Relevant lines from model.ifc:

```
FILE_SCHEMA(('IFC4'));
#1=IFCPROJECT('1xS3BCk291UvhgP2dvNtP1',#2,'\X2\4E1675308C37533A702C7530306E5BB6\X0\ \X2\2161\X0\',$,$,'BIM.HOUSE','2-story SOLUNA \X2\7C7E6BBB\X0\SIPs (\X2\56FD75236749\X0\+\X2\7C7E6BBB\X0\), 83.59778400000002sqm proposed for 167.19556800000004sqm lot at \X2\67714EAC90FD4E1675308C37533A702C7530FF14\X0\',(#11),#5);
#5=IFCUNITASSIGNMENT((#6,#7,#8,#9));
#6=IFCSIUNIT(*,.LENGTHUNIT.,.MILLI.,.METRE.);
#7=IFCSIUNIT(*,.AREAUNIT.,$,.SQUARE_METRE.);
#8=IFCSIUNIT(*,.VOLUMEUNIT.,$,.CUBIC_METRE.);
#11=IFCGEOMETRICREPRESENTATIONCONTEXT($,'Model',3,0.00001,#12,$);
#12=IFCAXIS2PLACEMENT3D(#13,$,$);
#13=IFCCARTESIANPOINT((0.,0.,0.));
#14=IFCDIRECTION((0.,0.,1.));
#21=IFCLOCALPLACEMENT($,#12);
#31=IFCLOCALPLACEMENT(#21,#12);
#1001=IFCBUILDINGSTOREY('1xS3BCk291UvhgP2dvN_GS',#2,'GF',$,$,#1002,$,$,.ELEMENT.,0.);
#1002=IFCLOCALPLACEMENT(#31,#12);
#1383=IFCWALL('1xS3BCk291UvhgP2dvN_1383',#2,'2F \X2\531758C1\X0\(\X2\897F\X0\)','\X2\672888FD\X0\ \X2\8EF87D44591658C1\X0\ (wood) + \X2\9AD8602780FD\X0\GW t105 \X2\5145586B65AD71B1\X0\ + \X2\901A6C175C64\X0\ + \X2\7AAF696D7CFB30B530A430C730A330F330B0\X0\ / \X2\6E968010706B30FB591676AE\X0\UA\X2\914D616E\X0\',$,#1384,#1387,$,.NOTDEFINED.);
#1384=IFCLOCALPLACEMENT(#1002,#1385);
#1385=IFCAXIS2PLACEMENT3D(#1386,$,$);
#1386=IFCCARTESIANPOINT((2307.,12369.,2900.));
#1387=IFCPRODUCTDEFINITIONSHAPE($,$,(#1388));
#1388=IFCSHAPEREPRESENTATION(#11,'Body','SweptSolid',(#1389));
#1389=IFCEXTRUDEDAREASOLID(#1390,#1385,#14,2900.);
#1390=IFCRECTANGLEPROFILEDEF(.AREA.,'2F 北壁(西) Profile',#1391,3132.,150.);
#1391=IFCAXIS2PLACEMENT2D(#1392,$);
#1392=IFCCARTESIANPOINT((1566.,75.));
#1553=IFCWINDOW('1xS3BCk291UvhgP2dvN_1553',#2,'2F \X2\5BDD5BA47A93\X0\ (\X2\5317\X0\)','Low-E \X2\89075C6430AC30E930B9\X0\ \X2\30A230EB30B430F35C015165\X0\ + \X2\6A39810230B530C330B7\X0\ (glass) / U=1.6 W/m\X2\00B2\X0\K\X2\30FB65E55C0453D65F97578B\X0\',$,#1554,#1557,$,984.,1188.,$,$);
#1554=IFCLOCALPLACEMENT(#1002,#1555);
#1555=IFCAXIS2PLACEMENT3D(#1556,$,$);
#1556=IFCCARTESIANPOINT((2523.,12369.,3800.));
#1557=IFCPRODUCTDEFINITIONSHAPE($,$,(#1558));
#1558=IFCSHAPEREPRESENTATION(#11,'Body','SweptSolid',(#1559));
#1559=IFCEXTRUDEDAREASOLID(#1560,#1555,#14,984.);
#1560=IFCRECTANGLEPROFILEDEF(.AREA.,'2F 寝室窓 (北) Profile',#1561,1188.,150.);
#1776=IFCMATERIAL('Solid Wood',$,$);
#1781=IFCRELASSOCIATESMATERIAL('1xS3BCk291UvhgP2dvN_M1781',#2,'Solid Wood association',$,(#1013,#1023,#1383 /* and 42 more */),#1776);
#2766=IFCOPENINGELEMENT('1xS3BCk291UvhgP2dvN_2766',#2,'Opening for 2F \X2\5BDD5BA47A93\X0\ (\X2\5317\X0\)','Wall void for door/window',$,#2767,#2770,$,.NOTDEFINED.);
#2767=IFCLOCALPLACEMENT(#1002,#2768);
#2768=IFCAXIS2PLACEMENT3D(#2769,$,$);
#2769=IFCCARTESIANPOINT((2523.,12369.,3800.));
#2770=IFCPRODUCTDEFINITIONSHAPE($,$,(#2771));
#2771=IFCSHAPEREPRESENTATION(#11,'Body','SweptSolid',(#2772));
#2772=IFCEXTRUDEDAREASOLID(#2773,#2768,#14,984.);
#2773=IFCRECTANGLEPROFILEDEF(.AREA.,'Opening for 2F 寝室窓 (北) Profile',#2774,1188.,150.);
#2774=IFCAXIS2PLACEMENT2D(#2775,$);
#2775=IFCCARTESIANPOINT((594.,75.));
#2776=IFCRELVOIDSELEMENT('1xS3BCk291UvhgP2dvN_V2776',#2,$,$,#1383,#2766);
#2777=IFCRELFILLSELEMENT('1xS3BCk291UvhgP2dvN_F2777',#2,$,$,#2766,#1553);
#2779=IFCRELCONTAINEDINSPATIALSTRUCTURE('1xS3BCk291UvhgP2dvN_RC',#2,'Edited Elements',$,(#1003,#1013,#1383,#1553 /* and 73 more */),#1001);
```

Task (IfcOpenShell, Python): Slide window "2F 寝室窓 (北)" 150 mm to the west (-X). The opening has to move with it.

```python
import ifcopenshell
import ifcopenshell.api.geometry
import ifcopenshell.util.placement

model = ifcopenshell.open("model.ifc")

window = model.by_guid("1xS3BCk291UvhgP2dvN_1553")
opening = window.FillsVoids[0].RelatingOpeningElement
wall = opening.VoidsElements[0].RelatingBuildingElement

wall_matrix = ifcopenshell.util.placement.get_local_placement(wall.ObjectPlacement)
shift = wall_matrix[:3, 0] * -150.0
before = ifcopenshell.util.placement.get_local_placement(window.ObjectPlacement)[:3, 3].copy()

# The window is not placed relative to its opening, so move both.
for product in (opening, window):
    matrix = ifcopenshell.util.placement.get_local_placement(product.ObjectPlacement)
    matrix[:3, 3] += shift
    ifcopenshell.api.geometry.edit_object_placement(model, product=product, matrix=matrix, is_si=False)

after = ifcopenshell.util.placement.get_local_placement(window.ObjectPlacement)[:3, 3]
print("window moved by", (after - before).round(3) + 0.0)

model.write("model-out.ifc")
```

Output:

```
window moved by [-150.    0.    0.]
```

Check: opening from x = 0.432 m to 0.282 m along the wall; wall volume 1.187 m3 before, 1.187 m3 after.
